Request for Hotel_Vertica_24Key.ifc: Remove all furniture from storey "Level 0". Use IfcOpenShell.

First a look at what the model holds.

```python
import ifcopenshell
import ifcopenshell.util.element

model = ifcopenshell.open("Hotel_Vertica_24Key.ifc")
print(model.schema)
storey = next(s for s in model.by_type("IfcBuildingStorey") if s.Name == "Level 0")
furniture = [e for e in ifcopenshell.util.element.get_decomposition(storey) if e.is_a("IfcFurnishingElement")]
seen = {}
for e in furniture:
    element_type = ifcopenshell.util.element.get_type(e)
    name = element_type.Name if element_type not in (None, e) else None
    seen[name] = seen.get(name, 0) + 1
for name, count in sorted(seen.items(), key=str):
    print(count, "x", name)
```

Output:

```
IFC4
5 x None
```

```python
import ifcopenshell
import ifcopenshell.api.root
import ifcopenshell.util.element

model = ifcopenshell.open("Hotel_Vertica_24Key.ifc")

storey = next(s for s in model.by_type("IfcBuildingStorey") if s.Name == "Level 0")
furniture = [e for e in ifcopenshell.util.element.get_decomposition(storey) if e.is_a("IfcFurnishingElement")]

for e in furniture:
    ifcopenshell.api.root.remove_product(model, product=e)
print(len(furniture), "removed")

model.write("Hotel_Vertica_24Key-out.ifc")
```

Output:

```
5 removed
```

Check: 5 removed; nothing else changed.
